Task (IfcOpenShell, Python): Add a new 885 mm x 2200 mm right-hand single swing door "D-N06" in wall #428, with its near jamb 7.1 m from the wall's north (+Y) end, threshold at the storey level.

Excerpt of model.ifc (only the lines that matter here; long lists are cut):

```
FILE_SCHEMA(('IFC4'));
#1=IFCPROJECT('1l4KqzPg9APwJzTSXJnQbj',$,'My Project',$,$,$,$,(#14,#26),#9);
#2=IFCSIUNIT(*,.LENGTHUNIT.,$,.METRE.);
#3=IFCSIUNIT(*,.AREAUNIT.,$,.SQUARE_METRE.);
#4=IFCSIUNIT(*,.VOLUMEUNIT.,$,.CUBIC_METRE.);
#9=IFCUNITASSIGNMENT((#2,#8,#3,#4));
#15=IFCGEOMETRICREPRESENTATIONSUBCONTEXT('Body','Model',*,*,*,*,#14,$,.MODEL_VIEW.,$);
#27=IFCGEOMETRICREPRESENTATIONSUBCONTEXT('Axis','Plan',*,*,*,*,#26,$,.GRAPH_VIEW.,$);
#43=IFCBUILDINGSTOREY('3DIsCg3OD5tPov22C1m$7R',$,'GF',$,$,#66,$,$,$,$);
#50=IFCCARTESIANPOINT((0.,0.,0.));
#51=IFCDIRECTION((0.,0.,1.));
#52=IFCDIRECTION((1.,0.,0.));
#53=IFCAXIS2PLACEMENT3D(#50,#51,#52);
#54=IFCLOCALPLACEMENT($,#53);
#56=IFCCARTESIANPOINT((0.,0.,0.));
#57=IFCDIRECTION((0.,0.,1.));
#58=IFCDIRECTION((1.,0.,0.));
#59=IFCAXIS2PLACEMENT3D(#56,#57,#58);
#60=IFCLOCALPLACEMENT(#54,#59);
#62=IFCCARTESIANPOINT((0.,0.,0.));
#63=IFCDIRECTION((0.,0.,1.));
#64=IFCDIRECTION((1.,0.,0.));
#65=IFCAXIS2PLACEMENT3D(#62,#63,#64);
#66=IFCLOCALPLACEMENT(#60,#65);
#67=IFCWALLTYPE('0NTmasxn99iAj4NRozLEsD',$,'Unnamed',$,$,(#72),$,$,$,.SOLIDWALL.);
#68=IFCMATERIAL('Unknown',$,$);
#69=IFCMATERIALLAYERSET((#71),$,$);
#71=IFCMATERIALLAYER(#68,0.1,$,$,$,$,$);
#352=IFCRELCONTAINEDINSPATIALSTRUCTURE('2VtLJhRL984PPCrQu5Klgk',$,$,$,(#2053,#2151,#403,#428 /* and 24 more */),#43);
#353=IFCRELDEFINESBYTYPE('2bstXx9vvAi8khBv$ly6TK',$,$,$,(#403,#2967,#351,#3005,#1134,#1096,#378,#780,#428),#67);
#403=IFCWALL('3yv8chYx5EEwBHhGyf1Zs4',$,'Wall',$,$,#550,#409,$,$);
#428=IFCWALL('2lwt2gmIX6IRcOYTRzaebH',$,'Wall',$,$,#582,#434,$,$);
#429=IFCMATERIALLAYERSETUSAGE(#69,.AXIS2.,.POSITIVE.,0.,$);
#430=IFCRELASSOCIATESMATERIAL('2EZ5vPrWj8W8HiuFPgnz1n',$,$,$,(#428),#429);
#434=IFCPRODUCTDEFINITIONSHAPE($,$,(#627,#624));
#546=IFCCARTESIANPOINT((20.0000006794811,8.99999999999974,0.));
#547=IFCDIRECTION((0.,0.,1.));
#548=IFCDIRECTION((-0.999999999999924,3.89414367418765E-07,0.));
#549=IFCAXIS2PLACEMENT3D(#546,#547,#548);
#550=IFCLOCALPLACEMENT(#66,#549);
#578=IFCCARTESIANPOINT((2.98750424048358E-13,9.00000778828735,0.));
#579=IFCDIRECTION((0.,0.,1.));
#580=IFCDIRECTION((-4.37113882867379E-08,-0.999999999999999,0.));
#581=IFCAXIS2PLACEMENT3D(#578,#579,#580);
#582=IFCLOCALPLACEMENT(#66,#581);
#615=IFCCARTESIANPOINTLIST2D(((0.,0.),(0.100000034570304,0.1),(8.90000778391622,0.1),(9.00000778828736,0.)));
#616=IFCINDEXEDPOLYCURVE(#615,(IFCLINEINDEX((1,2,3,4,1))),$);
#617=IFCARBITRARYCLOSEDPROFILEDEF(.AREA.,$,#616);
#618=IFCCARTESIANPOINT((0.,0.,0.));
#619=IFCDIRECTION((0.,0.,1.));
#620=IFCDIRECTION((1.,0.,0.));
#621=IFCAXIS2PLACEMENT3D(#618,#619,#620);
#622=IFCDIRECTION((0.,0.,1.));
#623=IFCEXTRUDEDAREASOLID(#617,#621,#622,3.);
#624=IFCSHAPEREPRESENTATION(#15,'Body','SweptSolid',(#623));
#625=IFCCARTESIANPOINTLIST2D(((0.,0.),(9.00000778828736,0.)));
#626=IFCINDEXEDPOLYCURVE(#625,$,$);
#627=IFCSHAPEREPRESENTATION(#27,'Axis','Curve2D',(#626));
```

```python
import numpy as np
import ifcopenshell
import ifcopenshell.api.feature
import ifcopenshell.api.geometry
import ifcopenshell.api.root
import ifcopenshell.api.spatial
import ifcopenshell.geom
import ifcopenshell.util.element
import ifcopenshell.util.placement
import ifcopenshell.util.representation
import ifcopenshell.util.shape
import ifcopenshell.util.unit

model = ifcopenshell.open("model.ifc")
unit_scale = ifcopenshell.util.unit.calculate_unit_scale(model)
settings = ifcopenshell.geom.settings()


def volume(element):
    """Net volume in cubic metres, openings subtracted."""
    shape = ifcopenshell.geom.create_shape(settings, element)
    return ifcopenshell.util.shape.get_volume(shape.geometry)


wall = model.by_id(428)
storey = ifcopenshell.util.element.get_container(wall, ifc_class="IfcBuildingStorey")
context = ifcopenshell.util.representation.get_context(model, "Model", "Body", "MODEL_VIEW")
before = volume(wall)

width, height, from_end, sill = 0.885, 2.2, 7.1, 0.0  # metres

# The wall runs along its own X axis, and the end named is its -X end.
wall_shape = ifcopenshell.geom.create_shape(settings, wall)
x, y, z = ifcopenshell.util.shape.get_vertices(wall_shape.geometry).T
start = x.min() + from_end
face, thickness = float(y.min()), float(y.max() - y.min())
wall_matrix = ifcopenshell.util.placement.get_local_placement(wall.ObjectPlacement)
level = ifcopenshell.util.placement.get_local_placement(storey.ObjectPlacement)[2, 3]


def in_wall(x, y):
    """Placement at x, y metres in the wall's axes, at sill height."""
    matrix = wall_matrix.copy()
    matrix[:, 3] = wall_matrix @ np.array([x / unit_scale, y / unit_scale, 0.0, 1.0])
    matrix[2, 3] = level + sill / unit_scale
    return matrix


# Opening: a box that overshoots both wall faces by 50 mm.
opening = ifcopenshell.api.root.create_entity(model, ifc_class="IfcOpeningElement", predefined_type="OPENING")
box = ifcopenshell.api.geometry.add_wall_representation(
    model, context=context, length=width, height=height, thickness=thickness + 0.1
)
ifcopenshell.api.geometry.assign_representation(model, product=opening, representation=box)
ifcopenshell.api.geometry.edit_object_placement(model, product=opening, matrix=in_wall(start, face - 0.05), is_si=False)
ifcopenshell.api.feature.add_feature(model, feature=opening, element=wall)

door = ifcopenshell.api.root.create_entity(model, ifc_class="IfcDoor", name="D-N06", predefined_type="DOOR")
door.OverallWidth, door.OverallHeight = width / unit_scale, height / unit_scale
door.OperationType = "SINGLE_SWING_RIGHT"
body = ifcopenshell.api.geometry.add_door_representation(
    model,
    context=context,
    overall_width=door.OverallWidth,
    overall_height=door.OverallHeight,
    operation_type="SINGLE_SWING_RIGHT",
    lining_properties={"LiningDepth": thickness / unit_scale, "ThresholdDepth": thickness / unit_scale},
)
ifcopenshell.api.geometry.assign_representation(model, product=door, representation=body)
ifcopenshell.api.spatial.assign_container(model, products=[door], relating_structure=storey)
ifcopenshell.api.feature.add_filling(model, opening=opening, element=door)

# The lining spans the wall, so the door starts at the wall face.
ifcopenshell.api.geometry.edit_object_placement(model, product=door, matrix=in_wall(start, face), is_si=False)

after = volume(wall)

print(f"wall volume {before:.3f} -> {after:.3f} m3")

model.write("model_updated.ifc")
```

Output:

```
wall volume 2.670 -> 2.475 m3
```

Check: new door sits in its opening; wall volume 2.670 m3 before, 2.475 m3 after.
